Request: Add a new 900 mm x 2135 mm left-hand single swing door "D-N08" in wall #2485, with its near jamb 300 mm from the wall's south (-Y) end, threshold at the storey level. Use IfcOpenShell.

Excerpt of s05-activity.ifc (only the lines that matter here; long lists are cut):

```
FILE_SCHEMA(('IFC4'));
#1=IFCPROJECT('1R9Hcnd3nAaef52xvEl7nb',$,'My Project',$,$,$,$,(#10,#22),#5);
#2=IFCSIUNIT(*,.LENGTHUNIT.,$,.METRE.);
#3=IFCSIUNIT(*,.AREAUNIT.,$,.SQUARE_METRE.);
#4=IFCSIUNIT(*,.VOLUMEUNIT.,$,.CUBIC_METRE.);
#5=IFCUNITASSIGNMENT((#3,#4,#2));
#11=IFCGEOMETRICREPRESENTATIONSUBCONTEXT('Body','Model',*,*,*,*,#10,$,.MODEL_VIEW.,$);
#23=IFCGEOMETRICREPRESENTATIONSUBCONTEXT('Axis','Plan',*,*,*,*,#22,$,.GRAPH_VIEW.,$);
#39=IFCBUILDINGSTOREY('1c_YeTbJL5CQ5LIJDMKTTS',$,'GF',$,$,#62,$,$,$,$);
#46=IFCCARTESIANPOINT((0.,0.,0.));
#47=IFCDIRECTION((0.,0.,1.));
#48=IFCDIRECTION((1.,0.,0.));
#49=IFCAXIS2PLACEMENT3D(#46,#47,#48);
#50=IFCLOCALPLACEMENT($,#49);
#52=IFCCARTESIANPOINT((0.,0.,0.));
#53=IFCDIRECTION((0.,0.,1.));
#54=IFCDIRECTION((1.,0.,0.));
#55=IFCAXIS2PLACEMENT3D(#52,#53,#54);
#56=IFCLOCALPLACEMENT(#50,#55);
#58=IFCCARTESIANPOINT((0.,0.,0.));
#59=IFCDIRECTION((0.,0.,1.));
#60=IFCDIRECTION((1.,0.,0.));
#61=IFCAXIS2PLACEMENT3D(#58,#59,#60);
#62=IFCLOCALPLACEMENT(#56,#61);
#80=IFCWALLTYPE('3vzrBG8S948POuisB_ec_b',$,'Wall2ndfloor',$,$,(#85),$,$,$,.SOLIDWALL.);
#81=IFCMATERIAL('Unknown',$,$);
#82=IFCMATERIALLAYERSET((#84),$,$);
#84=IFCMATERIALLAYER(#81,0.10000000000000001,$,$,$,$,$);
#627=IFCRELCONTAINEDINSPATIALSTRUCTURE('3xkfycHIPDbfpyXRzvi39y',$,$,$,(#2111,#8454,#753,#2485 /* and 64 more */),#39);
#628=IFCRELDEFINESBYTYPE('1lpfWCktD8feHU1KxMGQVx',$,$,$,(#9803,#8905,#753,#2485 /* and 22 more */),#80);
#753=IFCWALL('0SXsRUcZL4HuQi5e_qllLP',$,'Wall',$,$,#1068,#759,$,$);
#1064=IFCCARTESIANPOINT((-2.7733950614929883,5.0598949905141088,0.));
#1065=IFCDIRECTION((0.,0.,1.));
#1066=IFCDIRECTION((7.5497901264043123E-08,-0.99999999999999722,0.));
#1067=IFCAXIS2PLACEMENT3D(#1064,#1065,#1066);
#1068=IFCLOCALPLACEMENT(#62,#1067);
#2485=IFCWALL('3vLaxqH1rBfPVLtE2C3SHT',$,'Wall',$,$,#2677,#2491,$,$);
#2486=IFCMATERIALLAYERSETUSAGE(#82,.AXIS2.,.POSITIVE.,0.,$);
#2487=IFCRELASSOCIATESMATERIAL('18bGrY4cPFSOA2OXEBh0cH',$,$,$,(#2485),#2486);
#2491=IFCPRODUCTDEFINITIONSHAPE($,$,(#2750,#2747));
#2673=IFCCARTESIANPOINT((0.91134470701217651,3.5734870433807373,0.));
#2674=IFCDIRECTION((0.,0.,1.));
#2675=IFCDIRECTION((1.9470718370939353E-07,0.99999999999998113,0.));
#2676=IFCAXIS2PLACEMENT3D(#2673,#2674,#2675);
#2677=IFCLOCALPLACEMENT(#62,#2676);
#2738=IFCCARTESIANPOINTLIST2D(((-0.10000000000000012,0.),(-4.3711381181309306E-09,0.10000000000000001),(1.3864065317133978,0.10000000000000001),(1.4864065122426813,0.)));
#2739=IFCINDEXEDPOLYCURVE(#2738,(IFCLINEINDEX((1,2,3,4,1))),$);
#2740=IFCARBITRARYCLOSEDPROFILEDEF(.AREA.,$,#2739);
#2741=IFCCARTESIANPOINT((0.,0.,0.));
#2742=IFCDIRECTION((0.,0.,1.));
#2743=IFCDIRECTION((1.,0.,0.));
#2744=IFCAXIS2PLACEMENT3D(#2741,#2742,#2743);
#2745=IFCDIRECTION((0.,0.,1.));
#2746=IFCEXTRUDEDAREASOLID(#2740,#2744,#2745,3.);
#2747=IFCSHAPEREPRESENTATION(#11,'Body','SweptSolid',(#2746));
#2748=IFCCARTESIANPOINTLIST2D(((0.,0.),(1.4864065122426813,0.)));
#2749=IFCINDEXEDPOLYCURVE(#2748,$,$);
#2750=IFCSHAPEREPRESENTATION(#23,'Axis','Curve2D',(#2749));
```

```python
import numpy as np
import ifcopenshell
import ifcopenshell.api.feature
import ifcopenshell.api.geometry
import ifcopenshell.api.root
import ifcopenshell.api.spatial
import ifcopenshell.geom
import ifcopenshell.util.element
import ifcopenshell.util.placement
import ifcopenshell.util.representation
import ifcopenshell.util.shape
import ifcopenshell.util.unit

model = ifcopenshell.open("s05-activity.ifc")
unit_scale = ifcopenshell.util.unit.calculate_unit_scale(model)
settings = ifcopenshell.geom.settings()


def volume(element):
    """Net volume in cubic metres, openings subtracted."""
    shape = ifcopenshell.geom.create_shape(settings, element)
    return ifcopenshell.util.shape.get_volume(shape.geometry)


wall = model.by_guid("3vLaxqH1rBfPVLtE2C3SHT")
storey = ifcopenshell.util.element.get_container(wall, ifc_class="IfcBuildingStorey")
context = ifcopenshell.util.representation.get_context(model, "Model", "Body", "MODEL_VIEW")
before = volume(wall)

width, height, from_end, sill = 0.9, 2.135, 0.3, 0.0  # metres

# The wall runs along its own X axis, and the end named is its -X end.
wall_shape = ifcopenshell.geom.create_shape(settings, wall)
x, y, z = ifcopenshell.util.shape.get_vertices(wall_shape.geometry).T
start = x.min() + from_end
face, thickness = float(y.min()), float(y.max() - y.min())
wall_matrix = ifcopenshell.util.placement.get_local_placement(wall.ObjectPlacement)
level = ifcopenshell.util.placement.get_local_placement(storey.ObjectPlacement)[2, 3]


def in_wall(x, y):
    """Placement at x, y metres in the wall's axes, at sill height."""
    matrix = wall_matrix.copy()
    matrix[:, 3] = wall_matrix @ np.array([x / unit_scale, y / unit_scale, 0.0, 1.0])
    matrix[2, 3] = level + sill / unit_scale
    return matrix


# Opening: a box that overshoots both wall faces by 50 mm.
opening = ifcopenshell.api.root.create_entity(model, ifc_class="IfcOpeningElement", predefined_type="OPENING")
box = ifcopenshell.api.geometry.add_wall_representation(
    model, context=context, length=width, height=height, thickness=thickness + 0.1
)
ifcopenshell.api.geometry.assign_representation(model, product=opening, representation=box)
ifcopenshell.api.geometry.edit_object_placement(model, product=opening, matrix=in_wall(start, face - 0.05), is_si=False)
ifcopenshell.api.feature.add_feature(model, feature=opening, element=wall)

door = ifcopenshell.api.root.create_entity(model, ifc_class="IfcDoor", name="D-N08", predefined_type="DOOR")
door.OverallWidth, door.OverallHeight = width / unit_scale, height / unit_scale
door.OperationType = "SINGLE_SWING_LEFT"
body = ifcopenshell.api.geometry.add_door_representation(
    model,
    context=context,
    overall_width=door.OverallWidth,
    overall_height=door.OverallHeight,
    operation_type="SINGLE_SWING_LEFT",
    lining_properties={"LiningDepth": thickness / unit_scale, "ThresholdDepth": thickness / unit_scale},
)
ifcopenshell.api.geometry.assign_representation(model, product=door, representation=body)
ifcopenshell.api.spatial.assign_container(model, products=[door], relating_structure=storey)
ifcopenshell.api.feature.add_filling(model, opening=opening, element=door)

# The lining spans the wall, so the door starts at the wall face.
ifcopenshell.api.geometry.edit_object_placement(model, product=door, matrix=in_wall(start, face), is_si=False)

after = volume(wall)

print(f"wall volume {before:.3f} -> {after:.3f} m3")

model.write("s05-activity-out.ifc")
```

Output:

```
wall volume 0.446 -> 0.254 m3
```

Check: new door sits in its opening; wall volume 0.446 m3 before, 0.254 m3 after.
